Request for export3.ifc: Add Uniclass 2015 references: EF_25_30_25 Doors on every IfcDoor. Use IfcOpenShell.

First a look at what the model holds.

```python
import ifcopenshell

model = ifcopenshell.open("export3.ifc")
print(model.schema)
print("classifications:", [c.Name for c in model.by_type("IfcClassification")])
for ifc_class in ("IfcDoor", "IfcRoof", "IfcStair", "IfcWall", "IfcWindow"):
    print(ifc_class, len(model.by_type(ifc_class)))
```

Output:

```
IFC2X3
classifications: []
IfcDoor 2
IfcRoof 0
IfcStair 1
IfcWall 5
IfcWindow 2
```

```python
import ifcopenshell
import ifcopenshell.api.classification

model = ifcopenshell.open("export3.ifc")

# IFC2X3 requires Source and Edition and has no link from the project to the system.
system = model.create_entity("IfcClassification", Source="NBS", Edition="2015", Name="Uniclass 2015")

codes = {
    "IfcDoor": ("EF_25_30_25", "Doors"),
}
for ifc_class, (code, name) in codes.items():
    products = model.by_type(ifc_class)
    ifcopenshell.api.classification.add_reference(
        model, products=products, classification=system, identification=code, name=name
    )
    print(code, len(products))

model.write("export3_rev.ifc")
```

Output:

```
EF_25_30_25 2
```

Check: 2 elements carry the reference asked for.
